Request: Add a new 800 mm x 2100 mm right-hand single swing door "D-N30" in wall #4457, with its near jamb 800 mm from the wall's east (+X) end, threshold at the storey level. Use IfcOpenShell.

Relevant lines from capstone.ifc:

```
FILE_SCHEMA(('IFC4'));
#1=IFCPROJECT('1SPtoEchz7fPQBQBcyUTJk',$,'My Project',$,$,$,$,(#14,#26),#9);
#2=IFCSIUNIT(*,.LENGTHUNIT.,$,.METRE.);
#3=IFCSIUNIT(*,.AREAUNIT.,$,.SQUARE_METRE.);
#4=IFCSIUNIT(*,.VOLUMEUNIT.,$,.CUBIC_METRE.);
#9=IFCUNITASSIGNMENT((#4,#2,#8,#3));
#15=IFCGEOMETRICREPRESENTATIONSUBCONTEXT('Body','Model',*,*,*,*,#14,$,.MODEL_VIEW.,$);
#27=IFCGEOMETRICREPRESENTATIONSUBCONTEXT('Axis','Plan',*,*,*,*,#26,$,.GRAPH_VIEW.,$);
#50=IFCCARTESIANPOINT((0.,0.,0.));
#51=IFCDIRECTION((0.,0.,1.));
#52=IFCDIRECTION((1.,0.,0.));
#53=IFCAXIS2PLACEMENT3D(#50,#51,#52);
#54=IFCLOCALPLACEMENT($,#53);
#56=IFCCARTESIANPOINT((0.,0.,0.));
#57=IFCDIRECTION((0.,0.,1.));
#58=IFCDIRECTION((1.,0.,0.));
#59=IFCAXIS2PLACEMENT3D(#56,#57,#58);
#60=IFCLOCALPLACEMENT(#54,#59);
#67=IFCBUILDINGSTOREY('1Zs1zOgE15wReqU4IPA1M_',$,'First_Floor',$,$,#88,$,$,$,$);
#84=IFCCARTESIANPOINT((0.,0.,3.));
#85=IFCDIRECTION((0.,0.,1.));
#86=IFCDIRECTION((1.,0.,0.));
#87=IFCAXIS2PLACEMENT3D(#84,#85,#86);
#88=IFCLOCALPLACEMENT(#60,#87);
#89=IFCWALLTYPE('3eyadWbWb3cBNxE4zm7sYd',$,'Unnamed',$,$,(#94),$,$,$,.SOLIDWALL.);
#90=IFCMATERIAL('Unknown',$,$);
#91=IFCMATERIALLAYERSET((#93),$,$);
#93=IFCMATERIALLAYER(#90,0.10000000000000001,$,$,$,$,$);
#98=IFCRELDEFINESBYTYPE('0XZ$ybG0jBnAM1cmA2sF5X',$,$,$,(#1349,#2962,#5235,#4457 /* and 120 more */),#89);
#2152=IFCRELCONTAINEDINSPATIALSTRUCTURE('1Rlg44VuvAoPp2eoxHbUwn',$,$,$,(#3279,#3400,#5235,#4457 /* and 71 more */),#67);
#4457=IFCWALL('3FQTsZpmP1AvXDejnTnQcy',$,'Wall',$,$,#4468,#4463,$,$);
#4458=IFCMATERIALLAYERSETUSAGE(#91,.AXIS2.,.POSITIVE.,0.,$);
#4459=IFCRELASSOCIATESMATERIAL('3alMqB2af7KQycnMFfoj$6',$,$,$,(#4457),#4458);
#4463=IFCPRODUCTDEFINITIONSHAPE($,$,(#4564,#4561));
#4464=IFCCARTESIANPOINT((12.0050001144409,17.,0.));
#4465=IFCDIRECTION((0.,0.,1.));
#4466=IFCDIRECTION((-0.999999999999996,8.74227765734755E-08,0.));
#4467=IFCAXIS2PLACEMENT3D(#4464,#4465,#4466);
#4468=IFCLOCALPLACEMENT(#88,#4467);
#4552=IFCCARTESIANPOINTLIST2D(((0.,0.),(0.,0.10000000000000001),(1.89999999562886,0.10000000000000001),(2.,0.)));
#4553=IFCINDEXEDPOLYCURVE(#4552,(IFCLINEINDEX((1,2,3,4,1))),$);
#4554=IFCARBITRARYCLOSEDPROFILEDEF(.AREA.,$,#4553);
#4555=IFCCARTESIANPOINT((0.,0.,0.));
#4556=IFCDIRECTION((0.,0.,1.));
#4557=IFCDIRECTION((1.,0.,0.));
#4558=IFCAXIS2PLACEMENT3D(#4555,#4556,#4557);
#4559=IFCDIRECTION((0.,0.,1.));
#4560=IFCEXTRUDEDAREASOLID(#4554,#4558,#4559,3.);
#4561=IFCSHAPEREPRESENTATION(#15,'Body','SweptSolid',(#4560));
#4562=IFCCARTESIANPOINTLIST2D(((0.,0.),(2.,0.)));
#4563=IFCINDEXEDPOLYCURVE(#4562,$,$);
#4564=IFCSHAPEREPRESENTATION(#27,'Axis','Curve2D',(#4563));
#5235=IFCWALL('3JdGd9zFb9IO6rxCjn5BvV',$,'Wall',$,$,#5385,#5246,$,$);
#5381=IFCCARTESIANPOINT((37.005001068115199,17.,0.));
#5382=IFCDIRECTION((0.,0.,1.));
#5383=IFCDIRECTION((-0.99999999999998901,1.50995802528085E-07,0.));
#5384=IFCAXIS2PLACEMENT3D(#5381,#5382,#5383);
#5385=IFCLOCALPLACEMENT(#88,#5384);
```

```python
import numpy as np
import ifcopenshell
import ifcopenshell.api.feature
import ifcopenshell.api.geometry
import ifcopenshell.api.root
import ifcopenshell.api.spatial
import ifcopenshell.geom
import ifcopenshell.util.element
import ifcopenshell.util.placement
import ifcopenshell.util.representation
import ifcopenshell.util.shape
import ifcopenshell.util.unit

model = ifcopenshell.open("capstone.ifc")
unit_scale = ifcopenshell.util.unit.calculate_unit_scale(model)
settings = ifcopenshell.geom.settings()


def volume(element):
    """Net volume in cubic metres, openings subtracted."""
    shape = ifcopenshell.geom.create_shape(settings, element)
    return ifcopenshell.util.shape.get_volume(shape.geometry)


wall = model.by_guid("3FQTsZpmP1AvXDejnTnQcy")
storey = ifcopenshell.util.element.get_container(wall, ifc_class="IfcBuildingStorey")
context = ifcopenshell.util.representation.get_context(model, "Model", "Body", "MODEL_VIEW")
before = volume(wall)

width, height, from_end, sill = 0.8, 2.1, 0.8, 0.0  # metres

# The wall runs along its own X axis, and the end named is its -X end.
wall_shape = ifcopenshell.geom.create_shape(settings, wall)
x, y, z = ifcopenshell.util.shape.get_vertices(wall_shape.geometry).T
start = x.min() + from_end
face, thickness = float(y.min()), float(y.max() - y.min())
wall_matrix = ifcopenshell.util.placement.get_local_placement(wall.ObjectPlacement)
level = ifcopenshell.util.placement.get_local_placement(storey.ObjectPlacement)[2, 3]


def in_wall(x, y):
    """Placement at x, y metres in the wall's axes, at sill height."""
    matrix = wall_matrix.copy()
    matrix[:, 3] = wall_matrix @ np.array([x / unit_scale, y / unit_scale, 0.0, 1.0])
    matrix[2, 3] = level + sill / unit_scale
    return matrix


# Opening: a box that overshoots both wall faces by 50 mm.
opening = ifcopenshell.api.root.create_entity(model, ifc_class="IfcOpeningElement", predefined_type="OPENING")
box = ifcopenshell.api.geometry.add_wall_representation(
    model, context=context, length=width, height=height, thickness=thickness + 0.1
)
ifcopenshell.api.geometry.assign_representation(model, product=opening, representation=box)
ifcopenshell.api.geometry.edit_object_placement(model, product=opening, matrix=in_wall(start, face - 0.05), is_si=False)
ifcopenshell.api.feature.add_feature(model, feature=opening, element=wall)

door = ifcopenshell.api.root.create_entity(model, ifc_class="IfcDoor", name="D-N30", predefined_type="DOOR")
door.OverallWidth, door.OverallHeight = width / unit_scale, height / unit_scale
door.OperationType = "SINGLE_SWING_RIGHT"
body = ifcopenshell.api.geometry.add_door_representation(
    model,
    context=context,
    overall_width=door.OverallWidth,
    overall_height=door.OverallHeight,
    operation_type="SINGLE_SWING_RIGHT",
    lining_properties={"LiningDepth": thickness / unit_scale, "ThresholdDepth": thickness / unit_scale},
)
ifcopenshell.api.geometry.assign_representation(model, product=door, representation=body)
ifcopenshell.api.spatial.assign_container(model, products=[door], relating_structure=storey)
ifcopenshell.api.feature.add_filling(model, opening=opening, element=door)

# The lining spans the wall, so the door starts at the wall face.
ifcopenshell.api.geometry.edit_object_placement(model, product=door, matrix=in_wall(start, face), is_si=False)

after = volume(wall)

print(f"wall volume {before:.3f} -> {after:.3f} m3")

model.write("capstone-out.ifc")
```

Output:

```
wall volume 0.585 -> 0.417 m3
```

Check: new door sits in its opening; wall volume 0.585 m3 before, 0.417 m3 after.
